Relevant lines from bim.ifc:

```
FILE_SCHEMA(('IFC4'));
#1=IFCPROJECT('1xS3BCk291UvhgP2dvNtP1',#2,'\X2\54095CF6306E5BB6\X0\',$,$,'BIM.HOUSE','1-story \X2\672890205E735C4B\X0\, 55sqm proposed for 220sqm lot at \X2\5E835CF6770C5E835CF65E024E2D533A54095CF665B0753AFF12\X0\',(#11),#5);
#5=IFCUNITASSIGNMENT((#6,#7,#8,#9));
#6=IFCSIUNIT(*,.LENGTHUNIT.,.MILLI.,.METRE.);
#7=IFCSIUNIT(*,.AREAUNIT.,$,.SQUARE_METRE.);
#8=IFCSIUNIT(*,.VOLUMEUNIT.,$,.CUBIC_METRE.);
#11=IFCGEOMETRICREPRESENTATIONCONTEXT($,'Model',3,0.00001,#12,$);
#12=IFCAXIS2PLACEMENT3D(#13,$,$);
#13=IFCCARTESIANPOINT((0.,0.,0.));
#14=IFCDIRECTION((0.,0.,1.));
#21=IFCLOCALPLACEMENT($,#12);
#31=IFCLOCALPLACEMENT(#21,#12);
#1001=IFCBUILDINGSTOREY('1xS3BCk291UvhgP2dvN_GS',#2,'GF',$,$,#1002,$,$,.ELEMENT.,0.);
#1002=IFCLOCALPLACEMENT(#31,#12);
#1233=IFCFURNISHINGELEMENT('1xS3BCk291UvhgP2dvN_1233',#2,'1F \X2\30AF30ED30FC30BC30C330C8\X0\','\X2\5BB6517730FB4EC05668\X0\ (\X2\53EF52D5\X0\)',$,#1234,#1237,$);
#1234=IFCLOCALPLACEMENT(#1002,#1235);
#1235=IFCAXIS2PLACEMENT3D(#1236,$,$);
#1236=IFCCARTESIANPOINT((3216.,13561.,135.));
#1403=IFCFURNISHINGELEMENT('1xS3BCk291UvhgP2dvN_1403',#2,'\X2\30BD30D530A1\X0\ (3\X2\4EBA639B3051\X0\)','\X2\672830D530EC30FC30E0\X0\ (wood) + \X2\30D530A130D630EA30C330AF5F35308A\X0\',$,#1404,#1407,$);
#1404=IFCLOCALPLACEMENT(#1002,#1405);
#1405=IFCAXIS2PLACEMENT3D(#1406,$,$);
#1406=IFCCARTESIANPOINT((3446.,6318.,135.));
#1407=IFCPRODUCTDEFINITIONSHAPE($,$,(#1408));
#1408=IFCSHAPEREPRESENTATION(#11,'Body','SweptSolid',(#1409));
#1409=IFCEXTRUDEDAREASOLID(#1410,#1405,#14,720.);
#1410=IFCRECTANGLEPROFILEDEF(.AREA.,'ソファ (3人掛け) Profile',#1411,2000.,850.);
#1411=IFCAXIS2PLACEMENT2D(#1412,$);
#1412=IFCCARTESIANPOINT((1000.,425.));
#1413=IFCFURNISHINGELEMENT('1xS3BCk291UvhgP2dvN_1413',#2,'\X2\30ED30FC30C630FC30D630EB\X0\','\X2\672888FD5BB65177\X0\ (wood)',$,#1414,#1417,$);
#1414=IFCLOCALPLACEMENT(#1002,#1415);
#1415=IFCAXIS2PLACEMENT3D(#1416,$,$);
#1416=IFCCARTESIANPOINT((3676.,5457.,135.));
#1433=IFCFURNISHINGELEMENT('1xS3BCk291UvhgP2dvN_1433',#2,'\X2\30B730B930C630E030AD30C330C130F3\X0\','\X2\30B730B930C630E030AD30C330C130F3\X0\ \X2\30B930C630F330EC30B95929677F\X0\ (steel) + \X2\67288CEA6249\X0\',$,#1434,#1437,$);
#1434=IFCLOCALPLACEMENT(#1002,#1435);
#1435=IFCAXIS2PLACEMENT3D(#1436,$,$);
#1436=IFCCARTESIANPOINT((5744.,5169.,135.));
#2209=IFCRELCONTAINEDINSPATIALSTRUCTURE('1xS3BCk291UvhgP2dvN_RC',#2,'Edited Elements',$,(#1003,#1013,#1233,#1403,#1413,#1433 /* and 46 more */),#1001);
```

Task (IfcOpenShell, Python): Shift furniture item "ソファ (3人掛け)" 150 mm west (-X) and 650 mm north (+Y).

```python
import ifcopenshell
import ifcopenshell.api.geometry
import ifcopenshell.util.placement

model = ifcopenshell.open("bim.ifc")

item = model.by_guid("1xS3BCk291UvhgP2dvN_1403")
matrix = ifcopenshell.util.placement.get_local_placement(item.ObjectPlacement)
matrix[0, 3] -= 150.0
matrix[1, 3] += 650.0
ifcopenshell.api.geometry.edit_object_placement(model, product=item, matrix=matrix, is_si=False)

print(ifcopenshell.util.placement.get_local_placement(item.ObjectPlacement).round(3) + 0.0)

model.write("bim_edited.ifc")
```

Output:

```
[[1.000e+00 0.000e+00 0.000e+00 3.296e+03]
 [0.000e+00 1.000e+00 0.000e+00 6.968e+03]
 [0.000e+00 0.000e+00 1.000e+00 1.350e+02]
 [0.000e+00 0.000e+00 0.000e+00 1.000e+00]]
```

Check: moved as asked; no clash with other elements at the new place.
